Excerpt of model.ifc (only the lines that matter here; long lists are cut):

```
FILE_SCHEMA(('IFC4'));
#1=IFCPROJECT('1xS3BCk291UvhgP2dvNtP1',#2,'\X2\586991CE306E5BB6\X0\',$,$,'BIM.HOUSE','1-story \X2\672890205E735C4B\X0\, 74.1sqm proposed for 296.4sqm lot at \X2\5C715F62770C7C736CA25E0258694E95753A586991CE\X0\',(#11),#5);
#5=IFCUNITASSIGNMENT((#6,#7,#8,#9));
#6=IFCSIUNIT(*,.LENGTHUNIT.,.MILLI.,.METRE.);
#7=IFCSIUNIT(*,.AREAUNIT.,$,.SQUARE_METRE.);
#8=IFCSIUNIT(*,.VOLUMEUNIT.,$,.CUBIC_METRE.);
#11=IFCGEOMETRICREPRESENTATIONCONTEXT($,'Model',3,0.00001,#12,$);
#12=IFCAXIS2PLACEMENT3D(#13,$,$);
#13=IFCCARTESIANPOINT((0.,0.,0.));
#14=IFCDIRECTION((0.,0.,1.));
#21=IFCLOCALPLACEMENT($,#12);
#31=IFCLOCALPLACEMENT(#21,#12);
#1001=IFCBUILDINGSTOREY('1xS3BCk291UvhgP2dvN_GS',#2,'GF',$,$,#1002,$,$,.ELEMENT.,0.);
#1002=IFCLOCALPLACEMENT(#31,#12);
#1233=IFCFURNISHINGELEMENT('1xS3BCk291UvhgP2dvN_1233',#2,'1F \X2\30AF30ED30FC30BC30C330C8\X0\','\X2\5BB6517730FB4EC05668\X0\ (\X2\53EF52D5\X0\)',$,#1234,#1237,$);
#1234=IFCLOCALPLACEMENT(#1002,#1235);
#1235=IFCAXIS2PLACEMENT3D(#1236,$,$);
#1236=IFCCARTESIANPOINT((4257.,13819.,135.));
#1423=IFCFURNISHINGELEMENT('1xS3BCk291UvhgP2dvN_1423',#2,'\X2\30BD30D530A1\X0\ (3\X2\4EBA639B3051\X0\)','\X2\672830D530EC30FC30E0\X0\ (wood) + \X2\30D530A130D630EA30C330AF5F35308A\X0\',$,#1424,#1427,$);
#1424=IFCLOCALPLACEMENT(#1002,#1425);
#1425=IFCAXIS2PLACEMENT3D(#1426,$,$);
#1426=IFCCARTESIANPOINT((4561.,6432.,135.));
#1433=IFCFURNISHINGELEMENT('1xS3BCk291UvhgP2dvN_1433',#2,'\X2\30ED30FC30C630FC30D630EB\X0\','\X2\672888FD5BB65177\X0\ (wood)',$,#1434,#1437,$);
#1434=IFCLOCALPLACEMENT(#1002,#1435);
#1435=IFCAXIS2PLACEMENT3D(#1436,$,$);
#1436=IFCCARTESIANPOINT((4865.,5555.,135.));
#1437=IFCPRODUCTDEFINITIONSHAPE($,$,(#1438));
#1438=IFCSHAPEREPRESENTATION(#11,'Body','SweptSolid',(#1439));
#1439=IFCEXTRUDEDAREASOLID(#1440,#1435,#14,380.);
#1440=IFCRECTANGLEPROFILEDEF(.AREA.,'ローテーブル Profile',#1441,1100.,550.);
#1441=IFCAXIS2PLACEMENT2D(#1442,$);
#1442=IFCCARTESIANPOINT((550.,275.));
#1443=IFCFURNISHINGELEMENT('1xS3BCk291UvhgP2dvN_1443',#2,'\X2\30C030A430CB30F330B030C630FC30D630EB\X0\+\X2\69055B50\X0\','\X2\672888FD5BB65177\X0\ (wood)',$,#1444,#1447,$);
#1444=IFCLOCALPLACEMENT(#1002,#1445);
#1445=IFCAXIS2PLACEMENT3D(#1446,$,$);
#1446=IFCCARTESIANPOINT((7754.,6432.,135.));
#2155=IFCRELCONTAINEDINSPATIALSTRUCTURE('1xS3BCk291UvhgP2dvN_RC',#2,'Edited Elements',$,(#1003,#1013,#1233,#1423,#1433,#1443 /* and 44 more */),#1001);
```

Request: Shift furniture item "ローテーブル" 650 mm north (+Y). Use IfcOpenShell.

```python
import ifcopenshell
import ifcopenshell.api.geometry
import ifcopenshell.util.placement
import ifcopenshell.util.unit

model = ifcopenshell.open("model.ifc")
unit_scale = ifcopenshell.util.unit.calculate_unit_scale(model)

item = model.by_id(1433)
matrix = ifcopenshell.util.placement.get_local_placement(item.ObjectPlacement)
matrix[1, 3] += 0.65 / unit_scale
ifcopenshell.api.geometry.edit_object_placement(model, product=item, matrix=matrix, is_si=False)

print(ifcopenshell.util.placement.get_local_placement(item.ObjectPlacement).round(3) + 0.0)

model.write("model_edited.ifc")
```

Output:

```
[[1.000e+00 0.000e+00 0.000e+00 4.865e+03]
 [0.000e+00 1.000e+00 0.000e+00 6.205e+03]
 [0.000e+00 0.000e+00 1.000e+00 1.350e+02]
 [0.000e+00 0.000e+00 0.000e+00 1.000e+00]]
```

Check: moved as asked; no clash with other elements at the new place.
